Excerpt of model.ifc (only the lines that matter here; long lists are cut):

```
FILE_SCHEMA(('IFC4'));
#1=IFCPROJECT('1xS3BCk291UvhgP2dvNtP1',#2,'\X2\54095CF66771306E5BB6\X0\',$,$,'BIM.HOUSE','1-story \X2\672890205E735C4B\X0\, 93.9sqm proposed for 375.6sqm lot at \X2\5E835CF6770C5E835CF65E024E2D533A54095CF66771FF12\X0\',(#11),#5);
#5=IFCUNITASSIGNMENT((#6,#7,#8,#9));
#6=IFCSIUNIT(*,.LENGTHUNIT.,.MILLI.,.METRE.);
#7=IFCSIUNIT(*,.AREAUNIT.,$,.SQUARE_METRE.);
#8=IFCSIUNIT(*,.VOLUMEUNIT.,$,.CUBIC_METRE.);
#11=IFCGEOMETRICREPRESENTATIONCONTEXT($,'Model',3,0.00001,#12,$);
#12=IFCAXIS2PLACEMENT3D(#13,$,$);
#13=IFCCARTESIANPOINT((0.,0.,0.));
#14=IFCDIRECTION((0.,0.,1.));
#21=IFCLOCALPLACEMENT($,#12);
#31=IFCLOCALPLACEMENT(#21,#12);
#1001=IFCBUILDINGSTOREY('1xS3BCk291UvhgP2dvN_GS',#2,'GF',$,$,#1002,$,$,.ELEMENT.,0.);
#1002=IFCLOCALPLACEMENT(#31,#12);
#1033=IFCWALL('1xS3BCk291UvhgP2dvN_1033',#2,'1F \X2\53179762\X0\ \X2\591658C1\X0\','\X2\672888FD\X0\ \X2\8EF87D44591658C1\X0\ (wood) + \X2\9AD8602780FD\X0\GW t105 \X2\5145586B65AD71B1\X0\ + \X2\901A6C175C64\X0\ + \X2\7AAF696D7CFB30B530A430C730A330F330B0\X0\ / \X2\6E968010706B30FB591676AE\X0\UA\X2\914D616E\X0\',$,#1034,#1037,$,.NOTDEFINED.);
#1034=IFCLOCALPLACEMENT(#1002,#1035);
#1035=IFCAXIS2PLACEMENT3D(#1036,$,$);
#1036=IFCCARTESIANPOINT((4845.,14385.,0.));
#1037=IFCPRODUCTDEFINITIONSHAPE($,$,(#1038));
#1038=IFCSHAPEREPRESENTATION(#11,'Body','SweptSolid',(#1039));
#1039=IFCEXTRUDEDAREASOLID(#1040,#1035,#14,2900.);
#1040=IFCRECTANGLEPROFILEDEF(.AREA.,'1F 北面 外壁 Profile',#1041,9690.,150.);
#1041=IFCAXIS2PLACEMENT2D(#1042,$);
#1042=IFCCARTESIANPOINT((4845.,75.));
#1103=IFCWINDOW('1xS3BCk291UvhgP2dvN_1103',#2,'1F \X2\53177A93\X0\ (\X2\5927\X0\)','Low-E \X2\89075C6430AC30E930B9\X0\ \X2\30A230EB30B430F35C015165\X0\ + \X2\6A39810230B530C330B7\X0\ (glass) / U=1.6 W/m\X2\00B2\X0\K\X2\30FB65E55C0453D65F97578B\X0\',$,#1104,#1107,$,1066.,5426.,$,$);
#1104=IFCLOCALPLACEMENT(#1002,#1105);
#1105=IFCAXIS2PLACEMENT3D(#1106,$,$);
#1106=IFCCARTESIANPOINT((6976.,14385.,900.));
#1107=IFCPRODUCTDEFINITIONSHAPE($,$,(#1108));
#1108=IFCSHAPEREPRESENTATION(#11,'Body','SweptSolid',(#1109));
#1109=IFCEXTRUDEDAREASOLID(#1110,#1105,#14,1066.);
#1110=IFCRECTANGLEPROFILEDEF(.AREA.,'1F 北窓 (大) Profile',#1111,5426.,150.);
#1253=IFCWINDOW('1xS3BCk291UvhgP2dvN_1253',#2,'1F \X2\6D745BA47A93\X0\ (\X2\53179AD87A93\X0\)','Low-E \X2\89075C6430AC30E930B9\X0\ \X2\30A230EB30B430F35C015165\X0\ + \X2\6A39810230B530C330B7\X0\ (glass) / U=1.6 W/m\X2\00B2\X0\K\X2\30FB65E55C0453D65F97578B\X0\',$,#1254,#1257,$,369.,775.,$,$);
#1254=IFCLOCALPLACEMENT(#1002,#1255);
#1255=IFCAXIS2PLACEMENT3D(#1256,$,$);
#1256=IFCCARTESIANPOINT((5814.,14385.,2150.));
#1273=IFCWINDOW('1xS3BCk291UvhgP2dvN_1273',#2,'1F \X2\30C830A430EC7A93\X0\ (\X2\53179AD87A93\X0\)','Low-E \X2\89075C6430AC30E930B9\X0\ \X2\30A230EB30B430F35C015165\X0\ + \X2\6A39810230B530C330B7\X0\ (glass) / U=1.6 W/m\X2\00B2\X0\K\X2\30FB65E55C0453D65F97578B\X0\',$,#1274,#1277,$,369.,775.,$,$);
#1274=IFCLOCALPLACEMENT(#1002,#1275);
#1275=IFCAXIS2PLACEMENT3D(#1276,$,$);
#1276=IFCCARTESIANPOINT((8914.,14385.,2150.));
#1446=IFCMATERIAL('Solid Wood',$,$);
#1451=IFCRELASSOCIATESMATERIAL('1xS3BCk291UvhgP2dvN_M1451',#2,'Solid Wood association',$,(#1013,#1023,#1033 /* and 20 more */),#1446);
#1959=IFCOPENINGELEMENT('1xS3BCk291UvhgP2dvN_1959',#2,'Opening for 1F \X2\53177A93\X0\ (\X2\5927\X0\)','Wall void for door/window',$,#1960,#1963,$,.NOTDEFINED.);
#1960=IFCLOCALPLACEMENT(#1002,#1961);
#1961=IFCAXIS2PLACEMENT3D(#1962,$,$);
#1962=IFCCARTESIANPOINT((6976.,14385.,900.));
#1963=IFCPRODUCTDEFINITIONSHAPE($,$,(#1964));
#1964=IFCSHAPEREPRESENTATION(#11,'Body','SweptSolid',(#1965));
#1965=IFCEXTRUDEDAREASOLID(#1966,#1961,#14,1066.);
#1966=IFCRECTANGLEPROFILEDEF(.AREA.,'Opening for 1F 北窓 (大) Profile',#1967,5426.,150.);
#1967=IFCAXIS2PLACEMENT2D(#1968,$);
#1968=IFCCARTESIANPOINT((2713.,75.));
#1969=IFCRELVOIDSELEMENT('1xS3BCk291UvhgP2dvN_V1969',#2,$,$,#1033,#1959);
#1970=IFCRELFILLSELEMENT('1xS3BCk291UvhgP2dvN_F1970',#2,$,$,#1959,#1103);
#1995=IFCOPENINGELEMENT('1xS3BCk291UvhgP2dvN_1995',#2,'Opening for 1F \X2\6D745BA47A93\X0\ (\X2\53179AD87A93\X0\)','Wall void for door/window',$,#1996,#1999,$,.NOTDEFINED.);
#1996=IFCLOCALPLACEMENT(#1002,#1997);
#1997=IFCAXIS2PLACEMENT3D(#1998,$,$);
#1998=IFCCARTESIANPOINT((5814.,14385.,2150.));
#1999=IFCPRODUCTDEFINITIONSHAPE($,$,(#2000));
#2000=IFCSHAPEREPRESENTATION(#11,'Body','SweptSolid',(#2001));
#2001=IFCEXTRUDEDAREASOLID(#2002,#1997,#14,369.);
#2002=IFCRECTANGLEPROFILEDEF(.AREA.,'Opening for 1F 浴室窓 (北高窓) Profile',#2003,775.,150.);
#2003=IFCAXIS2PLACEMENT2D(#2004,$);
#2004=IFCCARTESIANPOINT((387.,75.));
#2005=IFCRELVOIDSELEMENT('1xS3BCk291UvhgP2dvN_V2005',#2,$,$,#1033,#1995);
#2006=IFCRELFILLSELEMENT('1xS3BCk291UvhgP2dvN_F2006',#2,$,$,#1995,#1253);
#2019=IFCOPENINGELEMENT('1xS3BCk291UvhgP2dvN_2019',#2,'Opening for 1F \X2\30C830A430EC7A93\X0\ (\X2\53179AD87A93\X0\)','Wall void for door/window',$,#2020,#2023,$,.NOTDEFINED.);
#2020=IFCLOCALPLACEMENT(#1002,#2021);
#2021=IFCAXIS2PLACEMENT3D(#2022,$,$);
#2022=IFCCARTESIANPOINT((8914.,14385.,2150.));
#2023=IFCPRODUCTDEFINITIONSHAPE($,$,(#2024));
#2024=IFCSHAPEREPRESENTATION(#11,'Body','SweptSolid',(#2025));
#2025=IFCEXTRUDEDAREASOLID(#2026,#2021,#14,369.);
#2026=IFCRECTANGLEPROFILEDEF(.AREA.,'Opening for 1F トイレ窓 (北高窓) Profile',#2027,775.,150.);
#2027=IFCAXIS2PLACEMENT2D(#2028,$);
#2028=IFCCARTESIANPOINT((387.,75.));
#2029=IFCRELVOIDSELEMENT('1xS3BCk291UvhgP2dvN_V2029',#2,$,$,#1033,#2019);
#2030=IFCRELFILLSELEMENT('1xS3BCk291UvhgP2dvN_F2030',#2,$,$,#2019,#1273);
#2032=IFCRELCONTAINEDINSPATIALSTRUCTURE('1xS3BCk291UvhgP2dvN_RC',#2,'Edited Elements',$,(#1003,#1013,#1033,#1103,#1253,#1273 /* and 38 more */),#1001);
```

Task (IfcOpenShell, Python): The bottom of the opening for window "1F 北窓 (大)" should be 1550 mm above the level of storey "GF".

```python
import numpy as np
import ifcopenshell
import ifcopenshell.api.geometry
import ifcopenshell.geom
import ifcopenshell.util.element
import ifcopenshell.util.placement
import ifcopenshell.util.shape
import ifcopenshell.util.unit

model = ifcopenshell.open("model.ifc")
unit_scale = ifcopenshell.util.unit.calculate_unit_scale(model)

window = model.by_guid("1xS3BCk291UvhgP2dvN_1103")
opening = window.FillsVoids[0].RelatingOpeningElement
storey = ifcopenshell.util.element.get_container(window, ifc_class="IfcBuildingStorey")
level = ifcopenshell.util.placement.get_local_placement(storey.ObjectPlacement)[2, 3]

# The opening's origin need not be at the sill, so measure its lowest point.
shape = ifcopenshell.geom.create_shape(ifcopenshell.geom.settings(), opening)
bottom = ifcopenshell.util.shape.get_shape_bottom_elevation(shape, shape.geometry) / unit_scale
dz = level + 1550.0 - bottom

shift = np.array([0.0, 0.0, dz])
# The window is not placed relative to its opening, so move both.
for product in (opening, window):
    matrix = ifcopenshell.util.placement.get_local_placement(product.ObjectPlacement)
    matrix[:3, 3] += shift
    ifcopenshell.api.geometry.edit_object_placement(model, product=product, matrix=matrix, is_si=False)

print(f"moved by {dz * unit_scale:+.3f} m")

model.write("model_rev.ifc")
```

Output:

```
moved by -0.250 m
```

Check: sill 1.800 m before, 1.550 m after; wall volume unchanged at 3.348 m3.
